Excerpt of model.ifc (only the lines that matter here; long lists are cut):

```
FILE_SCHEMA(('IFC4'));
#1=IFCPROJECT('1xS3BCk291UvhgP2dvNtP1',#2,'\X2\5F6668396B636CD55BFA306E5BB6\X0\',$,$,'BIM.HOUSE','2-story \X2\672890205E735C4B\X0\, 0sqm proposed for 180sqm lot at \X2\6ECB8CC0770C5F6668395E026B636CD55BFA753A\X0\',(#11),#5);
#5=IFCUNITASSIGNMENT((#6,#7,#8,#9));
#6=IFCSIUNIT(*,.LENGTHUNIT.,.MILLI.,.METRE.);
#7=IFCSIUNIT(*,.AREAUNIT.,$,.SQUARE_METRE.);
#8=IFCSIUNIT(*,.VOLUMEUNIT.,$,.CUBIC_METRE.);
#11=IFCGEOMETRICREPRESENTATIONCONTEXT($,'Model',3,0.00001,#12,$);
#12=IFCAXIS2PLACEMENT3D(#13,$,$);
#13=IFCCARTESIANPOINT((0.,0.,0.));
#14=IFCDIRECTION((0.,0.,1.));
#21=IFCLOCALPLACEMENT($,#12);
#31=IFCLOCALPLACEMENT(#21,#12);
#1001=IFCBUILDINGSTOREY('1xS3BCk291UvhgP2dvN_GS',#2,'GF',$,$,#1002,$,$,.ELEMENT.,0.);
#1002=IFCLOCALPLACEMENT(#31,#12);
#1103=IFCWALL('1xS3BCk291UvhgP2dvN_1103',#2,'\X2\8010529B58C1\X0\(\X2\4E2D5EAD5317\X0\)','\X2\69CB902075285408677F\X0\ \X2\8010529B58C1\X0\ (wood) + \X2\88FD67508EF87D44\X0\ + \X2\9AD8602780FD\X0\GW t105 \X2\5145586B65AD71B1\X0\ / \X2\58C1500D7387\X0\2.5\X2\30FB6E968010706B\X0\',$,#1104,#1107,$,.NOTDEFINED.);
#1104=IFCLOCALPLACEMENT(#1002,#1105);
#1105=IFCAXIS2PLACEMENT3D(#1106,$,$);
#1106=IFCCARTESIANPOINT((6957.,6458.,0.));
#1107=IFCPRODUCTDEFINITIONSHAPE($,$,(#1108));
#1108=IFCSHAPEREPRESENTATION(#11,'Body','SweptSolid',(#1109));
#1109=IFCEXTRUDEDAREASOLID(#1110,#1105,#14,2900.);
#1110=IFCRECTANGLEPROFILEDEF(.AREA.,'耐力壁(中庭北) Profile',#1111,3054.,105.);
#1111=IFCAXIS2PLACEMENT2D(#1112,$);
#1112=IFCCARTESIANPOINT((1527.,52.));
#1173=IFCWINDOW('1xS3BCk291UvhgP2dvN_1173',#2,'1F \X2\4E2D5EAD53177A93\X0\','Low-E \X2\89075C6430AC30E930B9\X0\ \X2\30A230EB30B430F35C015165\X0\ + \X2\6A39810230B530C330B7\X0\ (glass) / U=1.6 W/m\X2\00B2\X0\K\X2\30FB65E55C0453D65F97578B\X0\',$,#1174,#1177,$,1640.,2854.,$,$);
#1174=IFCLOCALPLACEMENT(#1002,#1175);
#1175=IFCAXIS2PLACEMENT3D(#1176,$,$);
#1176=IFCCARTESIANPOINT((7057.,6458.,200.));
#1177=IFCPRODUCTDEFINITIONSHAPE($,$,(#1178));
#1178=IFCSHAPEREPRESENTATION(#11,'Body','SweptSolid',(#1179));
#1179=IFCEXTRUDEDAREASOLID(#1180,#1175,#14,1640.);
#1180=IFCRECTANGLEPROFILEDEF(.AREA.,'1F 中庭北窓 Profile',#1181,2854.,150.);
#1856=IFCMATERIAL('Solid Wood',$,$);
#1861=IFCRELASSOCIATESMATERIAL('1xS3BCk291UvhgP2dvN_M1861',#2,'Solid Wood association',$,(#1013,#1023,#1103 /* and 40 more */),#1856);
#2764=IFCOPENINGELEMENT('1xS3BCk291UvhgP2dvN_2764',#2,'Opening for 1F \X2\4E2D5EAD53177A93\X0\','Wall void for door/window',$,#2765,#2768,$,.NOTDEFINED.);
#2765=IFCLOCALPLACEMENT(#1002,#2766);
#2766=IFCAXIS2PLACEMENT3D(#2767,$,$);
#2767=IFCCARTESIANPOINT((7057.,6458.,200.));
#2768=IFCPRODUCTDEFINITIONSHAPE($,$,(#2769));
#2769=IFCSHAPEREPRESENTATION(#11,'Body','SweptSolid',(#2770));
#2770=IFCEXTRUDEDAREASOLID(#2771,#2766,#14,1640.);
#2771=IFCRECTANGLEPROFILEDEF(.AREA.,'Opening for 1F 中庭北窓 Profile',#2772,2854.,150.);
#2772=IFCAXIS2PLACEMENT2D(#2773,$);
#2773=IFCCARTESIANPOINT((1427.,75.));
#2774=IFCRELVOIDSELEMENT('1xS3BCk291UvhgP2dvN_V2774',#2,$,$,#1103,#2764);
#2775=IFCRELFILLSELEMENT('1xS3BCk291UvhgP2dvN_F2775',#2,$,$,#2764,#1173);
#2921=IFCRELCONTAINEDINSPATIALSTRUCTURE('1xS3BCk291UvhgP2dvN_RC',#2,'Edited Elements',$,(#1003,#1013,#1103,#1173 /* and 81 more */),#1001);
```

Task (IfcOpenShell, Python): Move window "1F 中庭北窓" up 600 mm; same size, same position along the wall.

```python
import numpy as np
import ifcopenshell
import ifcopenshell.api.geometry
import ifcopenshell.util.placement
import ifcopenshell.util.unit

model = ifcopenshell.open("model.ifc")
unit_scale = ifcopenshell.util.unit.calculate_unit_scale(model)

window = model.by_guid("1xS3BCk291UvhgP2dvN_1173")
opening = window.FillsVoids[0].RelatingOpeningElement
dz = 0.6 / unit_scale

shift = np.array([0.0, 0.0, dz])
# The window is not placed relative to its opening, so move both.
for product in (opening, window):
    matrix = ifcopenshell.util.placement.get_local_placement(product.ObjectPlacement)
    matrix[:3, 3] += shift
    ifcopenshell.api.geometry.edit_object_placement(model, product=product, matrix=matrix, is_si=False)

print(f"moved by {dz * unit_scale:+.3f} m")

model.write("model_v2.ifc")
```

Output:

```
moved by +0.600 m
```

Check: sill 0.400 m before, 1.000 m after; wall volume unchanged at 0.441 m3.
